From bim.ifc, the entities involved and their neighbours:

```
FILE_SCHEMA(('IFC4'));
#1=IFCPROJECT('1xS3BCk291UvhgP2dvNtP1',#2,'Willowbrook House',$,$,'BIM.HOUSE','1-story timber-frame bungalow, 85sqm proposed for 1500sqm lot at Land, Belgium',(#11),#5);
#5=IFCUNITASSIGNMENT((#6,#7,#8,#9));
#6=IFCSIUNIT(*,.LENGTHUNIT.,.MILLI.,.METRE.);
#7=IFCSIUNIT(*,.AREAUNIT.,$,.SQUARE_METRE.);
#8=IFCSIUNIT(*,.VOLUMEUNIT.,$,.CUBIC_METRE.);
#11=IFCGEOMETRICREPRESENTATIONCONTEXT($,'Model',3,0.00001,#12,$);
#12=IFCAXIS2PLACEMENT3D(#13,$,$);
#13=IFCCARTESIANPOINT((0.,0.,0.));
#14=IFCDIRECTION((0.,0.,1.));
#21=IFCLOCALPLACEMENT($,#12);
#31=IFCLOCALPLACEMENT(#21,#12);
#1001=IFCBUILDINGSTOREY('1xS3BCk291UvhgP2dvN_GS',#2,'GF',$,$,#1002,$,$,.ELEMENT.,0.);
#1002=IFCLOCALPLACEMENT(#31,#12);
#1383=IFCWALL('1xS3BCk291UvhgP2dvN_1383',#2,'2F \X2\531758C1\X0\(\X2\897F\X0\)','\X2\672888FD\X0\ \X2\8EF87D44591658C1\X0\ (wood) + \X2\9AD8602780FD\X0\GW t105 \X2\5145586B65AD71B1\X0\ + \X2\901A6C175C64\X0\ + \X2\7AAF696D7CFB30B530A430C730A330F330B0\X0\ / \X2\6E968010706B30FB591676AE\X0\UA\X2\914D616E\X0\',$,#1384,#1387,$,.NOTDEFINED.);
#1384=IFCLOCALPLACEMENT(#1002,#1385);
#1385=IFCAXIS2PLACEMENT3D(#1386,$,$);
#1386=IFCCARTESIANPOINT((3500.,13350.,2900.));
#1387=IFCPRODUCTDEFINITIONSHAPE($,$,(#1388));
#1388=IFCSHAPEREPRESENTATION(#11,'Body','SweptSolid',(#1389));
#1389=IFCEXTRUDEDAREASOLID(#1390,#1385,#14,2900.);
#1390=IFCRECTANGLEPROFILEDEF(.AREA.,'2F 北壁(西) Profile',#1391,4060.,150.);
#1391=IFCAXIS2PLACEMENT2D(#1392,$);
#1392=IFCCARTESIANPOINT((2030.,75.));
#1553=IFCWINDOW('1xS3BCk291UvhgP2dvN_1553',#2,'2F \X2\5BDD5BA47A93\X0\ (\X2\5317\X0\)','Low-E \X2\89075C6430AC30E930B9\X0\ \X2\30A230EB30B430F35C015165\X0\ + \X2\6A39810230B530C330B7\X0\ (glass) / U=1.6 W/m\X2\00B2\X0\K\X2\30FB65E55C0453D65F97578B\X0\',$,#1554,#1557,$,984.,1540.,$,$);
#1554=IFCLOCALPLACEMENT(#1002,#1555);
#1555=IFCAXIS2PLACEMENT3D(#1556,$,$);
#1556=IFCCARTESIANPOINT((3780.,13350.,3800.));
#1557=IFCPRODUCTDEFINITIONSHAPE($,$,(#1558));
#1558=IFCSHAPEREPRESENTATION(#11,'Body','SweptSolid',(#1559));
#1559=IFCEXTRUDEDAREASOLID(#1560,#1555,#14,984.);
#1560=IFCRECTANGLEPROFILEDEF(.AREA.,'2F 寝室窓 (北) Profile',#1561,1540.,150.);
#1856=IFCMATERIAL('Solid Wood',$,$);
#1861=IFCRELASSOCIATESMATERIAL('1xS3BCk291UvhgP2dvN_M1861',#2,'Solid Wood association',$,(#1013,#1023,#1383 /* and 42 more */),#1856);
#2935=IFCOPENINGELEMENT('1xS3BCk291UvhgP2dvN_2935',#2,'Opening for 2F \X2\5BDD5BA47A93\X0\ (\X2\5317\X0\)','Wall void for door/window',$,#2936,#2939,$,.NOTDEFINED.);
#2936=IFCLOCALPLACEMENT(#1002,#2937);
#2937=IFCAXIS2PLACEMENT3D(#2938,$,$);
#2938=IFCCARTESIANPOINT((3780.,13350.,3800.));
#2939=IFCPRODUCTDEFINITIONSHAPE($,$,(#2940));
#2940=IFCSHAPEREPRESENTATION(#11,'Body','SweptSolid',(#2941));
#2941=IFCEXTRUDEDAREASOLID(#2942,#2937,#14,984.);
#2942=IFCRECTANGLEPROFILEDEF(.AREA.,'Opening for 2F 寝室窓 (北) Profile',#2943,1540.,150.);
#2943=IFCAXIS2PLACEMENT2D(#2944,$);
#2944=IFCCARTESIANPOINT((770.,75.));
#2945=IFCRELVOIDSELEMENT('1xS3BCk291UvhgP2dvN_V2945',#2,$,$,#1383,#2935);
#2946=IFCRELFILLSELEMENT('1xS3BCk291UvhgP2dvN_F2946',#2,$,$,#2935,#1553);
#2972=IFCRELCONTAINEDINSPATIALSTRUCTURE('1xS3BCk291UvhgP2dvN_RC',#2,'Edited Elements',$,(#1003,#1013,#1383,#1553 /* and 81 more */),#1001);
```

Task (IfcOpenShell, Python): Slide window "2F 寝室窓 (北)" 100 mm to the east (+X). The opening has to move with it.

```python
import ifcopenshell
import ifcopenshell.api.geometry
import ifcopenshell.util.placement
import ifcopenshell.util.unit

model = ifcopenshell.open("bim.ifc")
unit_scale = ifcopenshell.util.unit.calculate_unit_scale(model)

window = model.by_id(1553)
opening = window.FillsVoids[0].RelatingOpeningElement
wall = opening.VoidsElements[0].RelatingBuildingElement

wall_matrix = ifcopenshell.util.placement.get_local_placement(wall.ObjectPlacement)
shift = wall_matrix[:3, 0] * 0.1 / unit_scale
before = ifcopenshell.util.placement.get_local_placement(window.ObjectPlacement)[:3, 3].copy()

# The window is not placed relative to its opening, so move both.
for product in (opening, window):
    matrix = ifcopenshell.util.placement.get_local_placement(product.ObjectPlacement)
    matrix[:3, 3] += shift
    ifcopenshell.api.geometry.edit_object_placement(model, product=product, matrix=matrix, is_si=False)

after = ifcopenshell.util.placement.get_local_placement(window.ObjectPlacement)[:3, 3]
print("window moved by", (after - before).round(3) + 0.0)

model.write("bim_v2.ifc")
```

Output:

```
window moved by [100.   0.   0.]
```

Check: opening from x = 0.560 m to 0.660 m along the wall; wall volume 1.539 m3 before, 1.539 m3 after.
